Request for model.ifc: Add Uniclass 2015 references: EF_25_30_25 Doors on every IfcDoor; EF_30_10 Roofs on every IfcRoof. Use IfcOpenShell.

First a look at what the model holds.

```python
import ifcopenshell

model = ifcopenshell.open("model.ifc")
print(model.schema)
print("classifications:", [c.Name for c in model.by_type("IfcClassification")])
for ifc_class in ("IfcDoor", "IfcRoof", "IfcStair", "IfcWall", "IfcWindow"):
    print(ifc_class, len(model.by_type(ifc_class)))
```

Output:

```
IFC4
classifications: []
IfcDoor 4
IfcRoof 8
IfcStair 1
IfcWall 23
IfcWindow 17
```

```python
import ifcopenshell
import ifcopenshell.api.classification

model = ifcopenshell.open("model.ifc")

system = ifcopenshell.api.classification.add_classification(model, classification="Uniclass 2015")

codes = {
    "IfcDoor": ("EF_25_30_25", "Doors"),
    "IfcRoof": ("EF_30_10", "Roofs"),
}
for ifc_class, (code, name) in codes.items():
    products = model.by_type(ifc_class)
    ifcopenshell.api.classification.add_reference(
        model, products=products, classification=system, identification=code, name=name
    )
    print(code, len(products))

model.write("model_v2.ifc")
```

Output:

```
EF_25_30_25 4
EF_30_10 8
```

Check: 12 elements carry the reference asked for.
